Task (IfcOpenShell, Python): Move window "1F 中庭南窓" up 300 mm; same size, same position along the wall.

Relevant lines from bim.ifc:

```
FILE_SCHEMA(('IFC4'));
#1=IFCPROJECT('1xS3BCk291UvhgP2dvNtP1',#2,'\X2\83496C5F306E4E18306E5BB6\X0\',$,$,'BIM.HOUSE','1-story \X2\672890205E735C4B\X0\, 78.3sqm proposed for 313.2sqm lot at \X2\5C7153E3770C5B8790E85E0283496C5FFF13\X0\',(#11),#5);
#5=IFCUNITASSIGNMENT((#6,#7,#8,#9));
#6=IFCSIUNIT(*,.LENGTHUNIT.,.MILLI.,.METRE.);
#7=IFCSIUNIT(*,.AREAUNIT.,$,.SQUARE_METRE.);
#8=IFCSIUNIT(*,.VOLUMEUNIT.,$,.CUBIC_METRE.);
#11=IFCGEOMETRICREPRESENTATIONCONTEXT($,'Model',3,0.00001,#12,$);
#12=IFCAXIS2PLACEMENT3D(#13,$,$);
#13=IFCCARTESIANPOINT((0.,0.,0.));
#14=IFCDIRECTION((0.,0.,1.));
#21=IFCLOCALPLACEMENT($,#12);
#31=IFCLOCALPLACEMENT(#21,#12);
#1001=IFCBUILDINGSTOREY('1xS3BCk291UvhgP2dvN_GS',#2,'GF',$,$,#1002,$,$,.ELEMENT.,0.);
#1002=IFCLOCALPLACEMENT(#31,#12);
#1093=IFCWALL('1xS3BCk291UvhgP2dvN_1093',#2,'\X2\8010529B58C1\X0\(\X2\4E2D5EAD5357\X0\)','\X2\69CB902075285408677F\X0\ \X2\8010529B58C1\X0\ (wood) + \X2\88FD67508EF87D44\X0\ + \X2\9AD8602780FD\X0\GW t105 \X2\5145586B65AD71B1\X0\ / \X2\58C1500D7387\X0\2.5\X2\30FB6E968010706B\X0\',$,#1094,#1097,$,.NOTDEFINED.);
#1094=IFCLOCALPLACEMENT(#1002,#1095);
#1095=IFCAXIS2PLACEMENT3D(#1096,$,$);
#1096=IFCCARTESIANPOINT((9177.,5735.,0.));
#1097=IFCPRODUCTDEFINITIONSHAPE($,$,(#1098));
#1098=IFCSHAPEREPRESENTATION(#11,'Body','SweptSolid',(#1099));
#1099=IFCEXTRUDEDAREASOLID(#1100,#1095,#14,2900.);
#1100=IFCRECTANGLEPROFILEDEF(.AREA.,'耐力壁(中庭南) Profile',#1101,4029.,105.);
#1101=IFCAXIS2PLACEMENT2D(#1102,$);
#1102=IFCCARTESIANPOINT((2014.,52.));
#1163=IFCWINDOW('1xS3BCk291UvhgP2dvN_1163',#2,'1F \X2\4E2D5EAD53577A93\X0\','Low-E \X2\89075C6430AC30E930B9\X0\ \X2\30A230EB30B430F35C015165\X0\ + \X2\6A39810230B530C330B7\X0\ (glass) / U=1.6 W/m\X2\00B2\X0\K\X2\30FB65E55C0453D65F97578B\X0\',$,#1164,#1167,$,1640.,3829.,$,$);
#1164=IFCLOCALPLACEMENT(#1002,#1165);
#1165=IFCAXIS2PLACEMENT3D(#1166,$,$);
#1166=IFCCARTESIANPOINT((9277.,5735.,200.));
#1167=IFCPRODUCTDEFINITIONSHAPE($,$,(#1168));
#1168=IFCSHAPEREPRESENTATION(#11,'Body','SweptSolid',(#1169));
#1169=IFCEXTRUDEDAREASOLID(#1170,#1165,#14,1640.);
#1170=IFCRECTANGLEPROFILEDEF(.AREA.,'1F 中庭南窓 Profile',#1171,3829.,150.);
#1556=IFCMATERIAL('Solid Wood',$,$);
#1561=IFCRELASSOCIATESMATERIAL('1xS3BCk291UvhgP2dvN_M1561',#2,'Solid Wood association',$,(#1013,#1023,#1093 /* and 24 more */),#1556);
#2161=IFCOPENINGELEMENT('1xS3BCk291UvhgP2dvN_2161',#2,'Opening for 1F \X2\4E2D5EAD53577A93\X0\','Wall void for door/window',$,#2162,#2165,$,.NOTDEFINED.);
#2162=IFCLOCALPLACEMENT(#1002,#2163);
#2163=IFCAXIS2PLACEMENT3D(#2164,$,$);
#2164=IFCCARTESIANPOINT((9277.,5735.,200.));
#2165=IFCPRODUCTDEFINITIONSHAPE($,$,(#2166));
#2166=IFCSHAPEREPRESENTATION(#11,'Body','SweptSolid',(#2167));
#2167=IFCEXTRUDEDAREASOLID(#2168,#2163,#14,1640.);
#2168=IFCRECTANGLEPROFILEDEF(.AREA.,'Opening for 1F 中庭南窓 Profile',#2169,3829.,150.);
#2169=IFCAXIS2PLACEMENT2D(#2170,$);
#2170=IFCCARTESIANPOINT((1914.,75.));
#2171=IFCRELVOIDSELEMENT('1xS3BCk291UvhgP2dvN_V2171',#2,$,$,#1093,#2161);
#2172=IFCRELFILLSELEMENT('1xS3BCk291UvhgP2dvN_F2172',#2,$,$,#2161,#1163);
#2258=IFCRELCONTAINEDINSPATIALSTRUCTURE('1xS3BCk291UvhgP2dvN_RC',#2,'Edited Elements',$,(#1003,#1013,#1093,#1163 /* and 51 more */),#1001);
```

```python
import numpy as np
import ifcopenshell
import ifcopenshell.api.geometry
import ifcopenshell.util.placement
import ifcopenshell.util.unit

model = ifcopenshell.open("bim.ifc")
unit_scale = ifcopenshell.util.unit.calculate_unit_scale(model)

window = model.by_guid("1xS3BCk291UvhgP2dvN_1163")
opening = window.FillsVoids[0].RelatingOpeningElement
dz = 0.3 / unit_scale

shift = np.array([0.0, 0.0, dz])
# The window is not placed relative to its opening, so move both.
for product in (opening, window):
    matrix = ifcopenshell.util.placement.get_local_placement(product.ObjectPlacement)
    matrix[:3, 3] += shift
    ifcopenshell.api.geometry.edit_object_placement(model, product=product, matrix=matrix, is_si=False)

print(f"moved by {dz * unit_scale:+.3f} m")

model.write("bim_rev.ifc")
```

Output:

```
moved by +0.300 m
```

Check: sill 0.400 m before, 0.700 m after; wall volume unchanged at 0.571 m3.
